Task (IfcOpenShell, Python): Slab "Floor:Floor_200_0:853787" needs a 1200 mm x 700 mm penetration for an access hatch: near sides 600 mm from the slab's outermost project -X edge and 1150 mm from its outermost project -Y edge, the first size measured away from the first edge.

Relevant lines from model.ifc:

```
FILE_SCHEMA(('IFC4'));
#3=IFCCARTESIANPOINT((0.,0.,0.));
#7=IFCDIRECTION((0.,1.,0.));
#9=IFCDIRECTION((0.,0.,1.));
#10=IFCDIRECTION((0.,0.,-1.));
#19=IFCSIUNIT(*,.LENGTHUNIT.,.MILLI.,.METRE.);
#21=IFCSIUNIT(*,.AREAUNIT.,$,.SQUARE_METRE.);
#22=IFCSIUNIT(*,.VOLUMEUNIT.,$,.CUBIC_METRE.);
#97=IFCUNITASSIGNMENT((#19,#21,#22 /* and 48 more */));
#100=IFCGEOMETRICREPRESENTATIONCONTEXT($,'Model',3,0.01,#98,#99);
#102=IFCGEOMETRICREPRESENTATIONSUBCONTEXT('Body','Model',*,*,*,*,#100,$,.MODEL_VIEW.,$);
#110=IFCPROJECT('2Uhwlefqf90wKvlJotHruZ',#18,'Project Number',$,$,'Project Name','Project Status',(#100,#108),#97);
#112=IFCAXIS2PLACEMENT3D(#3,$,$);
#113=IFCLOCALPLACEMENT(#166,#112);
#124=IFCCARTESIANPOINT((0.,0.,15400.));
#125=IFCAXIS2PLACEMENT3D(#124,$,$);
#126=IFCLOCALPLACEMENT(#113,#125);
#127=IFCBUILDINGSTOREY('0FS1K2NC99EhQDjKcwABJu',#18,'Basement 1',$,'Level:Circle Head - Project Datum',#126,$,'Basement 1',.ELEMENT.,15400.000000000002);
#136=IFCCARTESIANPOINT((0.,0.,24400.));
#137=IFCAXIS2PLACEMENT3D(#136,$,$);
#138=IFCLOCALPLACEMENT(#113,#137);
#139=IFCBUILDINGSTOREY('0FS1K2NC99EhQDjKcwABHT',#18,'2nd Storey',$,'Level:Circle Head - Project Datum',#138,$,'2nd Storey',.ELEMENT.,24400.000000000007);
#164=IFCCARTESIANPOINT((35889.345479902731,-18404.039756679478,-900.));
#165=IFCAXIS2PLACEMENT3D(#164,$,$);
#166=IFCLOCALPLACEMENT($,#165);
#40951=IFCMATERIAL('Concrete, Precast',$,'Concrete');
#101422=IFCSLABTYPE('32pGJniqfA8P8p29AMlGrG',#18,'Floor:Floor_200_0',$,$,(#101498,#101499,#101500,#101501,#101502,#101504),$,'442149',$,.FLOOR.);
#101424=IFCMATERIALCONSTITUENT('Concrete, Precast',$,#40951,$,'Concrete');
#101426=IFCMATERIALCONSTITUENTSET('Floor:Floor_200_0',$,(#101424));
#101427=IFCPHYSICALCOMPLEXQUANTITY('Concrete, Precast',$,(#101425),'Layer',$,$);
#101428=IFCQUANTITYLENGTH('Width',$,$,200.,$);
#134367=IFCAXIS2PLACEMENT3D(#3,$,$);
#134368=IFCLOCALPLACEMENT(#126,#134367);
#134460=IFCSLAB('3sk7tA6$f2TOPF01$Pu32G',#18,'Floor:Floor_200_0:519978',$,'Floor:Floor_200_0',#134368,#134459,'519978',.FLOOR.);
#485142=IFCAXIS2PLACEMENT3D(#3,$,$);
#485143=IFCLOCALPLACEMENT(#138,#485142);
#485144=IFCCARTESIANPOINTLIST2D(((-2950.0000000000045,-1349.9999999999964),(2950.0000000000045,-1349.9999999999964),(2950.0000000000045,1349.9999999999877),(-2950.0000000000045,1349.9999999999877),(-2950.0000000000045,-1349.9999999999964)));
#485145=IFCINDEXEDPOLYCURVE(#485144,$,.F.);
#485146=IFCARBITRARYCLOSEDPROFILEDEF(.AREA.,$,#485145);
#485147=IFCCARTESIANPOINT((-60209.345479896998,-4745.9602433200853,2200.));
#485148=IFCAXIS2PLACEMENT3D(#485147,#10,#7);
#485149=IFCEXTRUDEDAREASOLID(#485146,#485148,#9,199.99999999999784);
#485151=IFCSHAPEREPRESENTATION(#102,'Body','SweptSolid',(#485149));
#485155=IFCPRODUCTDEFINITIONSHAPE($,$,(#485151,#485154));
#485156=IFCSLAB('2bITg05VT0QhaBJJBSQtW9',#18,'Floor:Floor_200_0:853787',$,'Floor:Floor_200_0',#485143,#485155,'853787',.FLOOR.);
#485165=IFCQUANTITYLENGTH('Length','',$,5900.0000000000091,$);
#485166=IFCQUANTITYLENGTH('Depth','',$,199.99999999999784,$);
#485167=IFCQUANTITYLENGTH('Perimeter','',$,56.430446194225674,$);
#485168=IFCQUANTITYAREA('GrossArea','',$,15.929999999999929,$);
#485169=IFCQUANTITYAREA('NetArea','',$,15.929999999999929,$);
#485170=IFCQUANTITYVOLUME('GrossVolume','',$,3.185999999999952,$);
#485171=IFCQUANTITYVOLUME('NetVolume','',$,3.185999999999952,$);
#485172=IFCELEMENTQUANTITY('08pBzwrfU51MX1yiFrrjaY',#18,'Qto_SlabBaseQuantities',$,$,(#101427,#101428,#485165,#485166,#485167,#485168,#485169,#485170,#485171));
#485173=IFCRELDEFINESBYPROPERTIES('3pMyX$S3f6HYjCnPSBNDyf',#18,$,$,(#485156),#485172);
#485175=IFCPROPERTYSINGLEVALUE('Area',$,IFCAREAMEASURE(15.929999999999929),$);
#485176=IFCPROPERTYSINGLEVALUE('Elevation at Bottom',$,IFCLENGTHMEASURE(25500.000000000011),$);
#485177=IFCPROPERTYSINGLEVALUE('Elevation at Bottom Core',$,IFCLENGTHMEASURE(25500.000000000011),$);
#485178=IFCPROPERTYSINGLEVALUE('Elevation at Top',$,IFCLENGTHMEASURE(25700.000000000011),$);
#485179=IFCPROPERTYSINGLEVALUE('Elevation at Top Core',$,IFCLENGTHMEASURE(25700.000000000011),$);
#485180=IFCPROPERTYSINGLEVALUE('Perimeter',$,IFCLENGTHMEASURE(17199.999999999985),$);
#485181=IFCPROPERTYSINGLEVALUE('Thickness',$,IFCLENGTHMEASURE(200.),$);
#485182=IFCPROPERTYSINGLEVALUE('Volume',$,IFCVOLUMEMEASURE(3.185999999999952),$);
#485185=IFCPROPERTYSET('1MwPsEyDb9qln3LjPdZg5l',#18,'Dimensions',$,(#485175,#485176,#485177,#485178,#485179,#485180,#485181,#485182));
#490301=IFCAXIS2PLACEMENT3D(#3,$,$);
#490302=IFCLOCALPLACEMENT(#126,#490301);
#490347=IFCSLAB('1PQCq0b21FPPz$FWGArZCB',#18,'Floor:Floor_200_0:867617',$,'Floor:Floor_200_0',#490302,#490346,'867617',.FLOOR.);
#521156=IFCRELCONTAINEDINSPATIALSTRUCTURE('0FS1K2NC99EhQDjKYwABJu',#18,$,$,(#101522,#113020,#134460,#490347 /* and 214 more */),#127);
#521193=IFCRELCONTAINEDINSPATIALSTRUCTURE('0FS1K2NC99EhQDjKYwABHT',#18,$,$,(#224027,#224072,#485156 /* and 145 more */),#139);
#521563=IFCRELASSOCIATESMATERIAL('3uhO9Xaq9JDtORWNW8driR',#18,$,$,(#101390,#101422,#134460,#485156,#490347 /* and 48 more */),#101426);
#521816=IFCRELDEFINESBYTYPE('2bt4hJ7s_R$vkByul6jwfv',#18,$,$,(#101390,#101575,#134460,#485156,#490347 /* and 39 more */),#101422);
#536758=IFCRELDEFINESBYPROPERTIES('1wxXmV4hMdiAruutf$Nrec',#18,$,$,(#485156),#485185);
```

```python
import numpy as np
import ifcopenshell
import ifcopenshell.api.feature
import ifcopenshell.api.geometry
import ifcopenshell.api.pset
import ifcopenshell.api.root
import ifcopenshell.geom
import ifcopenshell.util.element
import ifcopenshell.util.placement
import ifcopenshell.util.representation
import ifcopenshell.util.shape
import ifcopenshell.util.unit

model = ifcopenshell.open("model.ifc")
unit_scale = ifcopenshell.util.unit.calculate_unit_scale(model)
area_scale = ifcopenshell.util.unit.calculate_unit_scale(model, "AREAUNIT")
volume_scale = ifcopenshell.util.unit.calculate_unit_scale(model, "VOLUMEUNIT")
settings = ifcopenshell.geom.settings()


def volume(element):
    """Net volume in cubic metres, openings subtracted."""
    shape = ifcopenshell.geom.create_shape(settings, element)
    return ifcopenshell.util.shape.get_volume(shape.geometry)


slab = model.by_guid("2bITg05VT0QhaBJJBSQtW9")
before = volume(slab)

# Extent in the slab's own axes, in metres. The edges named are its -X and -Y sides.
slab_shape = ifcopenshell.geom.create_shape(settings, slab)
vertices = ifcopenshell.util.shape.get_vertices(slab_shape.geometry)
x_min, y_min, bottom = vertices.min(axis=0)
top = vertices[:, 2].max()

opening = ifcopenshell.api.root.create_entity(model, ifc_class="IfcOpeningElement", name="Access hatch opening", predefined_type="OPENING")
context = ifcopenshell.util.representation.get_context(model, "Model", "Body", "MODEL_VIEW")
width, depth = 1.2, 0.7
outline = [(0.0, 0.0), (width, 0.0), (width, depth), (0.0, depth), (0.0, 0.0)]
# Overshoot both faces by 50 mm so the cut is clean.
shape = ifcopenshell.api.geometry.add_slab_representation(
    model, context=context, depth=top - bottom + 0.1, polyline=outline
)
ifcopenshell.api.geometry.assign_representation(model, product=opening, representation=shape)

matrix = ifcopenshell.util.placement.get_local_placement(slab.ObjectPlacement)
matrix[:, 3] = matrix @ np.append(np.array([x_min + 0.6, y_min + 1.15, bottom - 0.05]) / unit_scale, 1.0)
ifcopenshell.api.geometry.edit_object_placement(model, product=opening, matrix=matrix, is_si=False)
ifcopenshell.api.feature.add_feature(model, feature=opening, element=slab)

after = volume(slab)

# Update the slab's stored quantities.
qto = model.by_id(ifcopenshell.util.element.get_pset(slab, "Qto_SlabBaseQuantities", should_inherit=False)["id"])
ifcopenshell.api.pset.edit_qto(model, qto=qto, properties={
    "NetArea": after / (top - bottom) / area_scale,
    "NetVolume": after / volume_scale,
})
pset = model.by_id(ifcopenshell.util.element.get_pset(slab, "Dimensions", should_inherit=False)["id"])
ifcopenshell.api.pset.edit_pset(model, pset=pset, properties={
    "Area": model.create_entity("IfcAreaMeasure", after / (top - bottom) / area_scale),
    "Volume": model.create_entity("IfcVolumeMeasure", after / volume_scale),
})

print(f"slab volume {before:.3f} -> {after:.3f} m3")

model.write("model_edited.ifc")
```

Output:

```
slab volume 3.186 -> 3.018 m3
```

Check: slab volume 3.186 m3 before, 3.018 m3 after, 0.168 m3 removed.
